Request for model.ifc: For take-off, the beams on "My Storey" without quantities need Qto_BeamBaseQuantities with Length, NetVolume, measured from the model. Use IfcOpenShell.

First a look at what the model holds.

```python
import ifcopenshell
import ifcopenshell.util.element
import ifcopenshell.util.unit

model = ifcopenshell.open("model.ifc")
print(model.schema)
for unit_type in ("LENGTHUNIT", "AREAUNIT", "VOLUMEUNIT"):
    print(unit_type, ifcopenshell.util.unit.calculate_unit_scale(model, unit_type))
storey = next(s for s in model.by_type("IfcBuildingStorey") if s.Name == "My Storey")
beams = [e for e in ifcopenshell.util.element.get_decomposition(storey) if e.is_a("IfcBeam")]
for e in sorted(beams, key=lambda e: e.id()):
    print(e.id(), e.is_a(), e.Name, list(ifcopenshell.util.element.get_psets(e, qtos_only=True)), sep=" | ")
```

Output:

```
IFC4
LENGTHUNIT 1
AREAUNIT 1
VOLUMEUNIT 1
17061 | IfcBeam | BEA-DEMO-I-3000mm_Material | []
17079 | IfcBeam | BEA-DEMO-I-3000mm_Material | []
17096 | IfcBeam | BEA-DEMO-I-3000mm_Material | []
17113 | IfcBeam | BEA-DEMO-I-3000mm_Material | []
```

```python
import ifcopenshell
import ifcopenshell.api.pset
import ifcopenshell.geom
import ifcopenshell.util.element
import ifcopenshell.util.shape
import ifcopenshell.util.unit

model = ifcopenshell.open("model.ifc")
unit_scale = ifcopenshell.util.unit.calculate_unit_scale(model)
volume_scale = ifcopenshell.util.unit.calculate_unit_scale(model, "VOLUMEUNIT")
settings = ifcopenshell.geom.settings()

storey = next(s for s in model.by_type("IfcBuildingStorey") if s.Name == "My Storey")
beams = [e for e in ifcopenshell.util.element.get_decomposition(storey) if e.is_a("IfcBeam")]

for e in sorted(beams, key=lambda e: e.id()):
    if ifcopenshell.util.element.get_psets(e, qtos_only=True, should_inherit=False):
        continue
    # Geometry comes back in metres, in the element's own axes.
    shape = ifcopenshell.geom.create_shape(settings, e)
    values = {
        "Length": ifcopenshell.util.shape.get_max_xyz(shape.geometry) / unit_scale,
        "NetVolume": ifcopenshell.util.shape.get_volume(shape.geometry) / volume_scale,
    }
    qto = ifcopenshell.api.pset.add_qto(model, product=e, name="Qto_BeamBaseQuantities")
    ifcopenshell.api.pset.edit_qto(model, qto=qto, properties=values)
    print(e.id(), {k: round(v, 3) for k, v in values.items()})

model.write("model-out.ifc")
```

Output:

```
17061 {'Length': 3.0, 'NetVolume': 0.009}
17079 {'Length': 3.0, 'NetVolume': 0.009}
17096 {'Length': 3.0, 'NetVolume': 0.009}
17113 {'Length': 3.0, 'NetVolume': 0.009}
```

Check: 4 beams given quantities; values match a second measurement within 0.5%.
